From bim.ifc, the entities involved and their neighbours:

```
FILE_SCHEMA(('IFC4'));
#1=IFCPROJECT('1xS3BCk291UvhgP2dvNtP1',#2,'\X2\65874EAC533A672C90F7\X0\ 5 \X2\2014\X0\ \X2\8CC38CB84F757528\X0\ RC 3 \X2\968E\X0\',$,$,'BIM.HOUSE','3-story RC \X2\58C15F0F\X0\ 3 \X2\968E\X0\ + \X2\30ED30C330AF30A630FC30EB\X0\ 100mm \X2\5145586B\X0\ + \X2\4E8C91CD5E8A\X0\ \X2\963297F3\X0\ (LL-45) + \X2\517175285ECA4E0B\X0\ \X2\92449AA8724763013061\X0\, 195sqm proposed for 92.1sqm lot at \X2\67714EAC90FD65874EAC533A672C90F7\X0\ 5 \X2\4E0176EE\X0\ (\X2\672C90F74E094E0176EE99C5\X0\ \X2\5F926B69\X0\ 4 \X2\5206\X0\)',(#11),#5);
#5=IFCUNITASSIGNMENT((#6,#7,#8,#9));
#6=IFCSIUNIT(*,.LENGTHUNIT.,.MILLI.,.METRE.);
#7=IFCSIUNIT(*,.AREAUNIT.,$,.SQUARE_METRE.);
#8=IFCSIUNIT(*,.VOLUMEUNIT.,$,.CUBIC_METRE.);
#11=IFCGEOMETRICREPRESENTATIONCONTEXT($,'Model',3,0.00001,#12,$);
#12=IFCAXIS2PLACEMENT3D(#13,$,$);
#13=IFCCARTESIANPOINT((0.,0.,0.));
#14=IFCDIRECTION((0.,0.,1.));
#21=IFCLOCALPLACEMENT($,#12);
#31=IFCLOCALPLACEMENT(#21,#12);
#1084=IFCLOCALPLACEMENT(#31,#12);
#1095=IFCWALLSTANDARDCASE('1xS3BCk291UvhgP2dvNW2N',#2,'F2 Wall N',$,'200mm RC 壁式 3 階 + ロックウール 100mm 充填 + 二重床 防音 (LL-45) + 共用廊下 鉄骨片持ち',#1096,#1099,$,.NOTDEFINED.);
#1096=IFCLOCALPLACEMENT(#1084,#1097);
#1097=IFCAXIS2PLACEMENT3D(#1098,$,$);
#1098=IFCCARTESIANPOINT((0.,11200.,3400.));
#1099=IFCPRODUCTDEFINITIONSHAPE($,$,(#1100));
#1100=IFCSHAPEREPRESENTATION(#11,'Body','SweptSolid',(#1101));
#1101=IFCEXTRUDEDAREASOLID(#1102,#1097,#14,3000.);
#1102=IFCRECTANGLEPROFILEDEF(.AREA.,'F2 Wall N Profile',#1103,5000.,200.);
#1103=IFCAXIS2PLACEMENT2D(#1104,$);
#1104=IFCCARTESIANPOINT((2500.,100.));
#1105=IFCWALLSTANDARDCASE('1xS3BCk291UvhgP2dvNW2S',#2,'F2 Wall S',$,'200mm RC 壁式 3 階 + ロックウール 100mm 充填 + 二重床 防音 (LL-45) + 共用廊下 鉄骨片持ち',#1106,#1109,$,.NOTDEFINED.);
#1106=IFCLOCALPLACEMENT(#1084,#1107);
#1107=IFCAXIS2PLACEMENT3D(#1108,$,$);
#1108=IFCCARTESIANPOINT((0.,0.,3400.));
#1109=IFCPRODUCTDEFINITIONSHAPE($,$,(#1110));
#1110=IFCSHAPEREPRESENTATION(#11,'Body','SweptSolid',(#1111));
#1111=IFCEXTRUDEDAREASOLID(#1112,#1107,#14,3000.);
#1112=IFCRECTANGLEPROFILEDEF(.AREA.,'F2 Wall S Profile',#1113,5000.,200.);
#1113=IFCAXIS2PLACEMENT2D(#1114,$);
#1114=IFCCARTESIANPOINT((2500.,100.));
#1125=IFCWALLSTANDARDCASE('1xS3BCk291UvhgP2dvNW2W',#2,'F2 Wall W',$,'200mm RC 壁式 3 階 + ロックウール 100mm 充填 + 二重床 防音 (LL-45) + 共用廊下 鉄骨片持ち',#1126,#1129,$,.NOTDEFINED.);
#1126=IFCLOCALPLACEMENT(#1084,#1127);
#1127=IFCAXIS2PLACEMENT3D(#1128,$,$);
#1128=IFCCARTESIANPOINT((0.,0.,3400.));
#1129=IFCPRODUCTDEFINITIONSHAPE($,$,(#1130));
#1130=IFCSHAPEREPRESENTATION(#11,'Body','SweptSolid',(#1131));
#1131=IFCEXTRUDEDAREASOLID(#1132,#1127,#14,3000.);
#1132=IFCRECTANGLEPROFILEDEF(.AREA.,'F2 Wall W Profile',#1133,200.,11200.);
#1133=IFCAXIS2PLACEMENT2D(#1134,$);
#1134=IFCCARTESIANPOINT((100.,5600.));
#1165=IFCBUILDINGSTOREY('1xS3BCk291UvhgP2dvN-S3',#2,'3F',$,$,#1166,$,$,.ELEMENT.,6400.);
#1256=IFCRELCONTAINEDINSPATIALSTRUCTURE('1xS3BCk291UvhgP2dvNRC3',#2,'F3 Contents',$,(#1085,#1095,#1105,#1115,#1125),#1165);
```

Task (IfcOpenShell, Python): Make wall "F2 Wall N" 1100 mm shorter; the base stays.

```python
import ifcopenshell
import ifcopenshell.geom
import ifcopenshell.util.shape

model = ifcopenshell.open("bim.ifc")
settings = ifcopenshell.geom.settings()


def volume(element):
    """Net volume in cubic metres, openings subtracted."""
    shape = ifcopenshell.geom.create_shape(settings, element)
    return ifcopenshell.util.shape.get_volume(shape.geometry)


wall = model.by_id(1095)
before = volume(wall)

body = next(r for r in wall.Representation.Representations if r.RepresentationIdentifier == "Body")
solid = body.Items[0]
old_height = solid.Depth
solid.Depth -= 1100.0
after = volume(wall)

print(f"height {old_height:g} -> {solid.Depth:g}, volume {before:.3f} -> {after:.3f} m3")

model.write("bim-out.ifc")
```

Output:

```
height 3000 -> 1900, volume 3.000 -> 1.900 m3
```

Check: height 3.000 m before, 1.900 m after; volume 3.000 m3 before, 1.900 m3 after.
